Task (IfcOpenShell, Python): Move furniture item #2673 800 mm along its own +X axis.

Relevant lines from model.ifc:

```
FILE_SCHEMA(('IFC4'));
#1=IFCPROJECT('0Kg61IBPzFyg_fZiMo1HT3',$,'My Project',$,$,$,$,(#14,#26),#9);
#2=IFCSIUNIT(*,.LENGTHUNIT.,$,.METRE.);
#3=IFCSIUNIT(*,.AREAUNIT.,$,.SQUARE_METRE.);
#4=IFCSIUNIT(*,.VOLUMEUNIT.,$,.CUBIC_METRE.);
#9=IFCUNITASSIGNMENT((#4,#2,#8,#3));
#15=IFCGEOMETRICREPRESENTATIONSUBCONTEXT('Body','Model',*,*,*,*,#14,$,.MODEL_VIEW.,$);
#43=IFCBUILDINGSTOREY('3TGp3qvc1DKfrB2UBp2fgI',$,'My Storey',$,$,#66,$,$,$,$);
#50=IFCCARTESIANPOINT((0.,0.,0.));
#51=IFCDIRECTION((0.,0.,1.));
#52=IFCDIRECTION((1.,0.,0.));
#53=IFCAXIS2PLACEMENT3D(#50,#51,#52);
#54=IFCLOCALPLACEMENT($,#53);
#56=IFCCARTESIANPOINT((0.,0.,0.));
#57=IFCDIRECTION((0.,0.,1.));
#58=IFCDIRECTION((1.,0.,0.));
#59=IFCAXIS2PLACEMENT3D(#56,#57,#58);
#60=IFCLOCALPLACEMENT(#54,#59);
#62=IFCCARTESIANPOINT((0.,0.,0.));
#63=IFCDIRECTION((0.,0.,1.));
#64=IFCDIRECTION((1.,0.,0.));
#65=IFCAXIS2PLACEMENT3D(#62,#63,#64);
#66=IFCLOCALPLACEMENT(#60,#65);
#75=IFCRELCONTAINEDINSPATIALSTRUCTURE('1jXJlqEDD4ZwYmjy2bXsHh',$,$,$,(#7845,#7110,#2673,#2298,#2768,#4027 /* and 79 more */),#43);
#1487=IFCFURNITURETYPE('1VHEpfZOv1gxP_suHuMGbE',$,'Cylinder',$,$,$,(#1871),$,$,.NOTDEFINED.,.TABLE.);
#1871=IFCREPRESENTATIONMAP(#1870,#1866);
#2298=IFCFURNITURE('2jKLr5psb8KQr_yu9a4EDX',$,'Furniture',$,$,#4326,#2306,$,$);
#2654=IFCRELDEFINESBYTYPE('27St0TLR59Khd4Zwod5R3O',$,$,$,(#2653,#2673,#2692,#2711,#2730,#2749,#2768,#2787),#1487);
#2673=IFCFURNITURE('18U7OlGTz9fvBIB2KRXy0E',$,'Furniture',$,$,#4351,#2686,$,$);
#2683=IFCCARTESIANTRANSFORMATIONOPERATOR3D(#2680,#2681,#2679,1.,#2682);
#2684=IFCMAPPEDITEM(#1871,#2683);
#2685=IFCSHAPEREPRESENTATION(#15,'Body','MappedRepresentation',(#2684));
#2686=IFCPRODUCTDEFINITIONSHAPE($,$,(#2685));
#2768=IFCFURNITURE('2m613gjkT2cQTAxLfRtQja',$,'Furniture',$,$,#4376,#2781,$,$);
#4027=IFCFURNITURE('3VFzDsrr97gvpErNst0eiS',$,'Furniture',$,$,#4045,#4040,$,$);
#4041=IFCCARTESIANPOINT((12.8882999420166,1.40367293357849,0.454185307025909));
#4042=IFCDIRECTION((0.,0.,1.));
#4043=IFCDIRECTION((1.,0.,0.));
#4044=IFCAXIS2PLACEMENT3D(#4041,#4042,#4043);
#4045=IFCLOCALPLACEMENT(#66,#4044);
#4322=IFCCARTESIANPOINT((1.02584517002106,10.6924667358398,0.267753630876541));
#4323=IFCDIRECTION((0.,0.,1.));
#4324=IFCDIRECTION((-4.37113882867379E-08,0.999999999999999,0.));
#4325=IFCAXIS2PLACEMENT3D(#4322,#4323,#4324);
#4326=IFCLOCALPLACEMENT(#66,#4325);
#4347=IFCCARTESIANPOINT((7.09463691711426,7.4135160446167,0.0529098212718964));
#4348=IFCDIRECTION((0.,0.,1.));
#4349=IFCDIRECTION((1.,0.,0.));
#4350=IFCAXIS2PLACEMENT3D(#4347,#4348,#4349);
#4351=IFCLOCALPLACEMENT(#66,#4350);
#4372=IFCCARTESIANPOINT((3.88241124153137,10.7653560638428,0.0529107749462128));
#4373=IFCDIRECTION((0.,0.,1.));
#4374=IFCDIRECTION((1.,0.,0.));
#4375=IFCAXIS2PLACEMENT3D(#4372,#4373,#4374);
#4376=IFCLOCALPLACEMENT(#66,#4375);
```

```python
import ifcopenshell
import ifcopenshell.api.geometry
import ifcopenshell.util.placement

model = ifcopenshell.open("model.ifc")

item = model.by_guid("18U7OlGTz9fvBIB2KRXy0E")
matrix = ifcopenshell.util.placement.get_local_placement(item.ObjectPlacement)
matrix[:3, 3] += matrix[:3, 0] * 0.8
ifcopenshell.api.geometry.edit_object_placement(model, product=item, matrix=matrix, is_si=False)

print(ifcopenshell.util.placement.get_local_placement(item.ObjectPlacement).round(3) + 0.0)

model.write("model_rev.ifc")
```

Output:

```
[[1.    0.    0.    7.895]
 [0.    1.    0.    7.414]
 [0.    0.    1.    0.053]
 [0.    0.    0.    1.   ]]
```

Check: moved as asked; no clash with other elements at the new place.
